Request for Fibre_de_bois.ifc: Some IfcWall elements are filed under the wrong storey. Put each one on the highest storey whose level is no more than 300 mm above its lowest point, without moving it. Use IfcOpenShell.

First a look at what the model holds.

```python
import ifcopenshell
import ifcopenshell.util.element
import ifcopenshell.util.placement

model = ifcopenshell.open("Fibre_de_bois.ifc")
print(model.schema)
for storey in model.by_type("IfcBuildingStorey"):
    level = ifcopenshell.util.placement.get_storey_elevation(storey)
    count = sum(e.is_a("IfcWall") for e in ifcopenshell.util.element.get_contained(storey))
    print(storey.id(), storey.Name, round(level, 3), count, sep=" | ")
```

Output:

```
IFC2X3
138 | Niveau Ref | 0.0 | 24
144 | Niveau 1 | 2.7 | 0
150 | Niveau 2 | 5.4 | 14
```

```python
import ifcopenshell
import ifcopenshell.api.spatial
import ifcopenshell.geom
import ifcopenshell.util.element
import ifcopenshell.util.placement
import ifcopenshell.util.shape
import ifcopenshell.util.unit

model = ifcopenshell.open("Fibre_de_bois.ifc")
unit_scale = ifcopenshell.util.unit.calculate_unit_scale(model)
settings = ifcopenshell.geom.settings()

levels = sorted(
    ((ifcopenshell.util.placement.get_storey_elevation(s) * unit_scale, s) for s in model.by_type("IfcBuildingStorey")),
    key=lambda pair: pair[0],
)

for e in model.by_type("IfcWall"):
    current = e.ContainedInStructure[0].RelatingStructure if e.ContainedInStructure else None
    if current is None or not current.is_a("IfcBuildingStorey"):
        continue
    shape = ifcopenshell.geom.create_shape(settings, e)
    bottom = ifcopenshell.util.shape.get_shape_bottom_elevation(shape, shape.geometry)
    below = [s for level, s in levels if level <= bottom + 0.3]
    storey = below[-1] if below else levels[0][1]
    if storey != current:
        # assign_container keeps the world position.
        ifcopenshell.api.spatial.assign_container(model, products=[e], relating_structure=storey)
        print(e.id(), current.Name, "->", storey.Name)

model.write("Fibre_de_bois_edited.ifc")
```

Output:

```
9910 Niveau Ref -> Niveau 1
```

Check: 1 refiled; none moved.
